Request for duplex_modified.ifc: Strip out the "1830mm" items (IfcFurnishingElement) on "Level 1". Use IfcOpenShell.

First a look at what the model holds.

```python
import ifcopenshell
import ifcopenshell.util.element

model = ifcopenshell.open("duplex_modified.ifc")
print(model.schema)
storey = next(s for s in model.by_type("IfcBuildingStorey") if s.Name == "Level 1")
furniture = [e for e in ifcopenshell.util.element.get_decomposition(storey) if e.is_a("IfcFurnishingElement")]
seen = {}
for e in furniture:
    element_type = ifcopenshell.util.element.get_type(e)
    name = element_type.Name if element_type not in (None, e) else None
    seen[name] = seen.get(name, 0) + 1
for name, count in sorted(seen.items(), key=str):
    print(count, "x", name)
```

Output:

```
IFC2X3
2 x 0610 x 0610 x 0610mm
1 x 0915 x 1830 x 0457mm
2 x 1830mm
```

```python
import ifcopenshell
import ifcopenshell.api.root
import ifcopenshell.util.element

model = ifcopenshell.open("duplex_modified.ifc")

storey = next(s for s in model.by_type("IfcBuildingStorey") if s.Name == "Level 1")
furniture = [e for e in ifcopenshell.util.element.get_decomposition(storey) if e.is_a("IfcFurnishingElement")]
targets = [e for e in furniture if (t := ifcopenshell.util.element.get_type(e)) not in (None, e) and t.Name == "1830mm"]

for e in targets:
    ifcopenshell.api.root.remove_product(model, product=e)
print(len(targets), "removed")

model.write("duplex_modified-out.ifc")
```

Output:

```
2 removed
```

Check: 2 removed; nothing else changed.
